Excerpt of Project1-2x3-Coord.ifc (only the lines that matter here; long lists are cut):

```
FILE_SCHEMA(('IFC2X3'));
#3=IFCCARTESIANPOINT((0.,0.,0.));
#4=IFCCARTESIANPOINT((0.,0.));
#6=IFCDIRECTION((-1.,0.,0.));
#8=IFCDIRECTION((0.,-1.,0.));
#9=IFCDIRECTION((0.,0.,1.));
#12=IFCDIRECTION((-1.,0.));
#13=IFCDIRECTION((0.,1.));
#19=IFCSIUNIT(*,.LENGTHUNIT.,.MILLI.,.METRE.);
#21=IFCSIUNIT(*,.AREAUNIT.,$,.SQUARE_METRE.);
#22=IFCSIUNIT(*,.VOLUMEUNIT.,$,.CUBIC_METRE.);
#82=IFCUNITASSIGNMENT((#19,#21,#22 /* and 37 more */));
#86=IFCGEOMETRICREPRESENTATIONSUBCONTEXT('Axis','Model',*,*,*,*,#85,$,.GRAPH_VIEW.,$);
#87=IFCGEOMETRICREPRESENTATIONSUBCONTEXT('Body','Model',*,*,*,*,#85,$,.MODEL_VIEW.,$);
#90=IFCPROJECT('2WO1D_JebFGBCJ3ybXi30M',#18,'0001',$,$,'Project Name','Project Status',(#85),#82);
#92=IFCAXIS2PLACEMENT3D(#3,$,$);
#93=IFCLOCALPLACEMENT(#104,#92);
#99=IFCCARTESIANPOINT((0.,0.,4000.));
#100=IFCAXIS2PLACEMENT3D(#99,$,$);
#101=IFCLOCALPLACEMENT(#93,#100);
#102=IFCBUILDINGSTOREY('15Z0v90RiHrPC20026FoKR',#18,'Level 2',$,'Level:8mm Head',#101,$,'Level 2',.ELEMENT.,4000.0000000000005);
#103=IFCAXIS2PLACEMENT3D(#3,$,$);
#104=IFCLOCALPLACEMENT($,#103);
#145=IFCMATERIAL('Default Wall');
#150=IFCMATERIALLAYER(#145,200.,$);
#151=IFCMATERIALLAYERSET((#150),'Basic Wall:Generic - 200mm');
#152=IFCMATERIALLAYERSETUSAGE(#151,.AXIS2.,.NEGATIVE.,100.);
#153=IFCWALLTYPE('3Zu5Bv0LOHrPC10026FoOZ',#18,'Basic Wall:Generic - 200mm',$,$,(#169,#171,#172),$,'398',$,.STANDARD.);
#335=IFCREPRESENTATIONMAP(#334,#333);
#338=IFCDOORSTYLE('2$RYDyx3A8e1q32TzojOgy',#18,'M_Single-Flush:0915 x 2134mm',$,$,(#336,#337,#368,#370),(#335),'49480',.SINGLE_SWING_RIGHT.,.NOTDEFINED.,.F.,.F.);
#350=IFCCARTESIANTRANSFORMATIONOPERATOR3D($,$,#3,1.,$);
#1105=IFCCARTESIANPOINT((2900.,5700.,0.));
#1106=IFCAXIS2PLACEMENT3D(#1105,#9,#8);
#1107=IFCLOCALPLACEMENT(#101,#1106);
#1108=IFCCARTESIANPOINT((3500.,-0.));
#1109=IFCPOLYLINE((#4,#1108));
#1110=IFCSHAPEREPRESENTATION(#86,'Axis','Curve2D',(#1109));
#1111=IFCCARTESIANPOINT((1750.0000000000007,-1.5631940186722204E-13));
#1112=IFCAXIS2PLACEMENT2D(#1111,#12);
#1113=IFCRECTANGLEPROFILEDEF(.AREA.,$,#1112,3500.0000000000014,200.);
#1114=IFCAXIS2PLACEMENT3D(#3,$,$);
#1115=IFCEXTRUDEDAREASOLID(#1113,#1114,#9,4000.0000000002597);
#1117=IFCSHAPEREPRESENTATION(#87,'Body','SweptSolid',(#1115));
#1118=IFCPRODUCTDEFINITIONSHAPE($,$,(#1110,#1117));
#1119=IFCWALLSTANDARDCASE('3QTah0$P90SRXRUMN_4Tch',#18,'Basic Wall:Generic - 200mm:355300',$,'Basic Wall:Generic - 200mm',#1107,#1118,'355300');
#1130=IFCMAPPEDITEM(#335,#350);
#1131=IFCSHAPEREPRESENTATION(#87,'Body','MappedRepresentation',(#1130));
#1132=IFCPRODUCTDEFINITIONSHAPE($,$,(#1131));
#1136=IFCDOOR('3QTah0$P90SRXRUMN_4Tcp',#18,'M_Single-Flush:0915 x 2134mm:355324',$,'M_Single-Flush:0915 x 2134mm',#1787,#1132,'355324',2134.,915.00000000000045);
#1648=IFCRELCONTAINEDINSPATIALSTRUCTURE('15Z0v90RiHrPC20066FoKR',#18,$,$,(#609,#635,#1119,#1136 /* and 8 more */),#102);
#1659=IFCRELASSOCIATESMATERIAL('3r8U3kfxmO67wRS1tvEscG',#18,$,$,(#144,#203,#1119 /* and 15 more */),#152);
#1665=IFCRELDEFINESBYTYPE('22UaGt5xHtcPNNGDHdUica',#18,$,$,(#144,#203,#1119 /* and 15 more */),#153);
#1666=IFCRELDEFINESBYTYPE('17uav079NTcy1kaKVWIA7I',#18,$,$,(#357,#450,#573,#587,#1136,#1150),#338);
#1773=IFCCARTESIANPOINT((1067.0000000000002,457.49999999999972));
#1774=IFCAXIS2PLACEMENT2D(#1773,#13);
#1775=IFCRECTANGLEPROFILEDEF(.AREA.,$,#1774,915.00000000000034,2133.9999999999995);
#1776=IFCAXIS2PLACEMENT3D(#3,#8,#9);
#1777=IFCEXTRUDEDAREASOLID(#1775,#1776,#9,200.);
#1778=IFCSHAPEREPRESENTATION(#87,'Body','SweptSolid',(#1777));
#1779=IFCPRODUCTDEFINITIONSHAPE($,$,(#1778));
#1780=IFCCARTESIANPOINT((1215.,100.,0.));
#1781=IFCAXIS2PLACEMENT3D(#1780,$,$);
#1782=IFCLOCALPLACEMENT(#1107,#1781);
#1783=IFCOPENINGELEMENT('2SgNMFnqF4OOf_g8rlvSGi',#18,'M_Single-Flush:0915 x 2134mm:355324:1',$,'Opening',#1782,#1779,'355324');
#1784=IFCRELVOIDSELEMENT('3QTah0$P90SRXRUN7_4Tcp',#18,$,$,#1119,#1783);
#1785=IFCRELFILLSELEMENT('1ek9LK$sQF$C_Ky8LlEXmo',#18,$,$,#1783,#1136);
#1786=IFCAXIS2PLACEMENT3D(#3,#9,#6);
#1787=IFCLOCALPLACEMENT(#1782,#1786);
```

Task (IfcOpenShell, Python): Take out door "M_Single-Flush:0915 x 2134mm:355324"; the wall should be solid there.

```python
import ifcopenshell
import ifcopenshell.api.feature
import ifcopenshell.api.root
import ifcopenshell.geom
import ifcopenshell.util.shape

model = ifcopenshell.open("Project1-2x3-Coord.ifc")
settings = ifcopenshell.geom.settings()


def volume(element):
    """Net volume in cubic metres, openings subtracted."""
    shape = ifcopenshell.geom.create_shape(settings, element)
    return ifcopenshell.util.shape.get_volume(shape.geometry)


door = model.by_guid("3QTah0$P90SRXRUMN_4Tcp")
opening = door.FillsVoids[0].RelatingOpeningElement
wall = opening.VoidsElements[0].RelatingBuildingElement
before = volume(wall)

ifcopenshell.api.root.remove_product(model, product=door)
ifcopenshell.api.feature.remove_feature(model, feature=opening)

after = volume(wall)

print(f"wall volume {before:.3f} -> {after:.3f} m3")

model.write("Project1-2x3-Coord_edited.ifc")
```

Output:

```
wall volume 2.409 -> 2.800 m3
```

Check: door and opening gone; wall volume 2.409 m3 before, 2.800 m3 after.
